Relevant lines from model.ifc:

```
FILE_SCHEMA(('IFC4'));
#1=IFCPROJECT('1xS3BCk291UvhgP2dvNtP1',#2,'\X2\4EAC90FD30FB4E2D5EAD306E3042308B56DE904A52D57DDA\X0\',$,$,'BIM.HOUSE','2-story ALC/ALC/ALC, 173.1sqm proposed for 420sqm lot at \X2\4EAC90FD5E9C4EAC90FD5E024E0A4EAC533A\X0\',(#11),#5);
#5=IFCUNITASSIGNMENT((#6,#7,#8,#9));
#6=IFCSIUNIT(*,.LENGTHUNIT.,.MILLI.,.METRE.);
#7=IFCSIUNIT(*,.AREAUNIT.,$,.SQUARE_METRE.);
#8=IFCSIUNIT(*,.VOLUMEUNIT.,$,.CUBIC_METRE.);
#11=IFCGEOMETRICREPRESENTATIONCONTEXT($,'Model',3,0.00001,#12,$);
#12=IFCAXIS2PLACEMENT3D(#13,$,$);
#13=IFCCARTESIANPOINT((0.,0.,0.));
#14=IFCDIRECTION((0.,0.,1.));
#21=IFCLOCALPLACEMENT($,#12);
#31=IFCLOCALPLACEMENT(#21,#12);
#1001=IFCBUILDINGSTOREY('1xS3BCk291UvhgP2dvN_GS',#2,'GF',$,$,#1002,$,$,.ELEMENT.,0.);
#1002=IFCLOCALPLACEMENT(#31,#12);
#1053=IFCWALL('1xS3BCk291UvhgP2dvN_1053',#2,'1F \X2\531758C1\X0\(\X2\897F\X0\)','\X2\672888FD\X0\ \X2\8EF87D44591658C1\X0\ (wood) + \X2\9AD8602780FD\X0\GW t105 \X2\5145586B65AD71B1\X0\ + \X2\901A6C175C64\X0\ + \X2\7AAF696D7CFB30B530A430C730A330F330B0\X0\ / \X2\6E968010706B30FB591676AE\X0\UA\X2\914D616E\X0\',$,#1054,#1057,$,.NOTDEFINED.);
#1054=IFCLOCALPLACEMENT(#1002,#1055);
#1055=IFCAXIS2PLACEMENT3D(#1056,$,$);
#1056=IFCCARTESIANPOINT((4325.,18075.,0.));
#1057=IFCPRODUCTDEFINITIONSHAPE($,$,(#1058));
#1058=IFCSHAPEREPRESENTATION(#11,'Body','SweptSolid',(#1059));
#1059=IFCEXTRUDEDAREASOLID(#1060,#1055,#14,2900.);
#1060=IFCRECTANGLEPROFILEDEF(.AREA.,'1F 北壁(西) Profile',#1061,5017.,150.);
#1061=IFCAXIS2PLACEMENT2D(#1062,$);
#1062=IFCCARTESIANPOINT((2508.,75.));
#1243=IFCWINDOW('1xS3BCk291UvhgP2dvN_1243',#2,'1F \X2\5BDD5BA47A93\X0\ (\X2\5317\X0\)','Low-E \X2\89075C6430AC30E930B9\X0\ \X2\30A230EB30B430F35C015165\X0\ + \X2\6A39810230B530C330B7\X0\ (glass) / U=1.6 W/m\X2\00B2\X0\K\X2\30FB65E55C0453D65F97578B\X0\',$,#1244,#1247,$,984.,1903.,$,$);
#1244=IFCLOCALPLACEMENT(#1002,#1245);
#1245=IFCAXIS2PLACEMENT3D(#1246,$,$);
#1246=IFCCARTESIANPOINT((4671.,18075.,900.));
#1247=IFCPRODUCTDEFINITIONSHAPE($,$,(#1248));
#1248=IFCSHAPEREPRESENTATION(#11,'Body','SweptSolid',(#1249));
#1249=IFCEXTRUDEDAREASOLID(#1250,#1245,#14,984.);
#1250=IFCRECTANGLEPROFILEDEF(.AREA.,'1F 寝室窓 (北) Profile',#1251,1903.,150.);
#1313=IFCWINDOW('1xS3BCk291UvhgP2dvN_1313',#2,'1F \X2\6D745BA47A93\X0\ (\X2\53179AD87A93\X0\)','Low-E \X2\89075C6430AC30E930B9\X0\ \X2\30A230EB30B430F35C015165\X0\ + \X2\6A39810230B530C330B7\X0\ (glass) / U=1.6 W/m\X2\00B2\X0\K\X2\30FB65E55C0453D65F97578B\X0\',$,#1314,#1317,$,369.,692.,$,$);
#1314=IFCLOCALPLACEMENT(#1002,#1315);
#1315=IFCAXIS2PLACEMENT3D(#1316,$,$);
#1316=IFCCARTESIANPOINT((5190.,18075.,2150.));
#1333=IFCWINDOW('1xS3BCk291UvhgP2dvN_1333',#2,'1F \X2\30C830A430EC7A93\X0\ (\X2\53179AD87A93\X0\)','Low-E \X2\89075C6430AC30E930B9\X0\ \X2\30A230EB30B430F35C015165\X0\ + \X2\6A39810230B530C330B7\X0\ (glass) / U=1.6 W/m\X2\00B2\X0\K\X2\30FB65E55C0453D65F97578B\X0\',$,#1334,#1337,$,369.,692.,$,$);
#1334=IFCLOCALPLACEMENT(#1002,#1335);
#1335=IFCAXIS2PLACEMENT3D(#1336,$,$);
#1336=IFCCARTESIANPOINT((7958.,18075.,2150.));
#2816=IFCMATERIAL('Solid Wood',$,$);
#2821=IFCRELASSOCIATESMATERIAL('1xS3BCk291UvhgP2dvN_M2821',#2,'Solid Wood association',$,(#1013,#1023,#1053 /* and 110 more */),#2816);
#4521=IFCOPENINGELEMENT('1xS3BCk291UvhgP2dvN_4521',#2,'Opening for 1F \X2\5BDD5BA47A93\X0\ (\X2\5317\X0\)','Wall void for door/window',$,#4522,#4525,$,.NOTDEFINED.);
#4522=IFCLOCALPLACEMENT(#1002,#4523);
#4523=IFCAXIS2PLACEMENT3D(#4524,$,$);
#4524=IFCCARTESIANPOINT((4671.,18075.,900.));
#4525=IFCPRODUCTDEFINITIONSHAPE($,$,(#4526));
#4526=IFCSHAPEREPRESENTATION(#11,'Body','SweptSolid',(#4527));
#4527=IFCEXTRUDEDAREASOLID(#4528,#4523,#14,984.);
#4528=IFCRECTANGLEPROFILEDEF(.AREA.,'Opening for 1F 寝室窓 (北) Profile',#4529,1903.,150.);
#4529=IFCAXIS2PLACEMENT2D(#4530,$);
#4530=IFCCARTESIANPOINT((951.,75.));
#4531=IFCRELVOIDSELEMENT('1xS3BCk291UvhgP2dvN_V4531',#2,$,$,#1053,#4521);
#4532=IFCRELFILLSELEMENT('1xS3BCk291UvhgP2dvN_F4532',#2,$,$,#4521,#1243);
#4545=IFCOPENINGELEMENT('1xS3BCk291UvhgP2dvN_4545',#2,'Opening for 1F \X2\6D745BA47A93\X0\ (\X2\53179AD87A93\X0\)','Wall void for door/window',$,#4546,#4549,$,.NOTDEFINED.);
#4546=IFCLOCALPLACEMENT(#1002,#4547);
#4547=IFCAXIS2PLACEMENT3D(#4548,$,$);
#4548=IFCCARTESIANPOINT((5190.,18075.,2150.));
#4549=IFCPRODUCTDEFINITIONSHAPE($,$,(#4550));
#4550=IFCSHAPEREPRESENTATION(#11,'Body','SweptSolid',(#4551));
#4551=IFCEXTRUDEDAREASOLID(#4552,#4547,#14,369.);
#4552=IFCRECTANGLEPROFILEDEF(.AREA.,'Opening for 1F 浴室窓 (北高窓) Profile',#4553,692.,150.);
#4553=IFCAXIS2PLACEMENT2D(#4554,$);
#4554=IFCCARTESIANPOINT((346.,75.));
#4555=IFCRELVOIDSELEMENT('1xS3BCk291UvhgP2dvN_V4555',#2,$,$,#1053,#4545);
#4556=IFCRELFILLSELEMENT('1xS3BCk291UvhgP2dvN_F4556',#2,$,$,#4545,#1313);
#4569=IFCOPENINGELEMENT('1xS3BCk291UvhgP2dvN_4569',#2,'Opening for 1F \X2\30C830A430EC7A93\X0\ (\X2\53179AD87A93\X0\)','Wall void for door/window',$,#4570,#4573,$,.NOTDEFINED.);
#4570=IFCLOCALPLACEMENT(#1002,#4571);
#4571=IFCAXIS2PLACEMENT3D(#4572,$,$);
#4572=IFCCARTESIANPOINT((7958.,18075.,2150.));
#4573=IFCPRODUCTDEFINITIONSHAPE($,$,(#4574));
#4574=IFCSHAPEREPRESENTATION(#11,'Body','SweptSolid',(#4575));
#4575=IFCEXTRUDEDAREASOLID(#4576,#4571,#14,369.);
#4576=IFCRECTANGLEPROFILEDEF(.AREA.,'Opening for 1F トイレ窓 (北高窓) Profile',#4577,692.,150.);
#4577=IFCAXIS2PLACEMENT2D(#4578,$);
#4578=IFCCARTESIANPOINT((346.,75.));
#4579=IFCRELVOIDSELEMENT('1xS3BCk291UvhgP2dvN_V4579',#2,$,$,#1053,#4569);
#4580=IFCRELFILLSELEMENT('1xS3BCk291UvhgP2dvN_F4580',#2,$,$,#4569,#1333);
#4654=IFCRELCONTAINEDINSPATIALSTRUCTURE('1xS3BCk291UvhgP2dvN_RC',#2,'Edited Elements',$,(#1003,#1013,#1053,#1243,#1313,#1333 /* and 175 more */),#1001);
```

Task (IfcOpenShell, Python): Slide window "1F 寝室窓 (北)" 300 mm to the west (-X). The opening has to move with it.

```python
import ifcopenshell
import ifcopenshell.api.geometry
import ifcopenshell.util.placement
import ifcopenshell.util.unit

model = ifcopenshell.open("model.ifc")
unit_scale = ifcopenshell.util.unit.calculate_unit_scale(model)

window = model.by_guid("1xS3BCk291UvhgP2dvN_1243")
opening = window.FillsVoids[0].RelatingOpeningElement
wall = opening.VoidsElements[0].RelatingBuildingElement

wall_matrix = ifcopenshell.util.placement.get_local_placement(wall.ObjectPlacement)
shift = wall_matrix[:3, 0] * -0.3 / unit_scale
before = ifcopenshell.util.placement.get_local_placement(window.ObjectPlacement)[:3, 3].copy()

# The window is not placed relative to its opening, so move both.
for product in (opening, window):
    matrix = ifcopenshell.util.placement.get_local_placement(product.ObjectPlacement)
    matrix[:3, 3] += shift
    ifcopenshell.api.geometry.edit_object_placement(model, product=product, matrix=matrix, is_si=False)

after = ifcopenshell.util.placement.get_local_placement(window.ObjectPlacement)[:3, 3]
print("window moved by", (after - before).round(3) + 0.0)

model.write("model_updated.ifc")
```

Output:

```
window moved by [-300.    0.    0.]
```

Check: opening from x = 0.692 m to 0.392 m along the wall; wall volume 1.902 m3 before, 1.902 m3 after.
